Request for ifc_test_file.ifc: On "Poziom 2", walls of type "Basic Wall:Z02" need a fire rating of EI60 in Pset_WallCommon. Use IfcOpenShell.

First a look at what the model holds.

```python
import ifcopenshell
import ifcopenshell.util.element

model = ifcopenshell.open("ifc_test_file.ifc")
print(model.schema)
storey = next(s for s in model.by_type("IfcBuildingStorey") if s.Name == "Poziom 2")
walls = [e for e in ifcopenshell.util.element.get_decomposition(storey) if e.is_a("IfcWall")]
seen = {}
for e in walls:
    element_type = ifcopenshell.util.element.get_type(e)
    key = (element_type.Name if element_type != e and element_type else None, ifcopenshell.util.element.get_pset(e, "Pset_WallCommon", "FireRating"))
    seen[key] = seen.get(key, 0) + 1
for (name, value), count in sorted(seen.items(), key=str):
    print(count, "x", name, "|", value)
```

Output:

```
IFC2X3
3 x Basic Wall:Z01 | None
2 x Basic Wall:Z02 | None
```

```python
import ifcopenshell
import ifcopenshell.api.pset
import ifcopenshell.util.element

model = ifcopenshell.open("ifc_test_file.ifc")

storey = next(s for s in model.by_type("IfcBuildingStorey") if s.Name == "Poziom 2")
walls = [e for e in ifcopenshell.util.element.get_decomposition(storey) if e.is_a("IfcWall")]

count = 0
for e in walls:
    element_type = ifcopenshell.util.element.get_type(e)
    if element_type in (None, e) or element_type.Name != "Basic Wall:Z02":
        continue
    found = ifcopenshell.util.element.get_pset(e, "Pset_WallCommon", should_inherit=False)
    if found:
        pset = model.by_id(found["id"])
        if len(ifcopenshell.util.element.get_elements_by_pset(pset)) > 1:
            pset = ifcopenshell.api.pset.unshare_pset(model, products=[e], pset=pset)[0]
    else:
        pset = ifcopenshell.api.pset.add_pset(model, product=e, name="Pset_WallCommon")
    ifcopenshell.api.pset.edit_pset(model, pset=pset, properties={"FireRating": "EI60"})
    count += 1

print(count, "walls updated")

model.write("ifc_test_file_edited.ifc")
```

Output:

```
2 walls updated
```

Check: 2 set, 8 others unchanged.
